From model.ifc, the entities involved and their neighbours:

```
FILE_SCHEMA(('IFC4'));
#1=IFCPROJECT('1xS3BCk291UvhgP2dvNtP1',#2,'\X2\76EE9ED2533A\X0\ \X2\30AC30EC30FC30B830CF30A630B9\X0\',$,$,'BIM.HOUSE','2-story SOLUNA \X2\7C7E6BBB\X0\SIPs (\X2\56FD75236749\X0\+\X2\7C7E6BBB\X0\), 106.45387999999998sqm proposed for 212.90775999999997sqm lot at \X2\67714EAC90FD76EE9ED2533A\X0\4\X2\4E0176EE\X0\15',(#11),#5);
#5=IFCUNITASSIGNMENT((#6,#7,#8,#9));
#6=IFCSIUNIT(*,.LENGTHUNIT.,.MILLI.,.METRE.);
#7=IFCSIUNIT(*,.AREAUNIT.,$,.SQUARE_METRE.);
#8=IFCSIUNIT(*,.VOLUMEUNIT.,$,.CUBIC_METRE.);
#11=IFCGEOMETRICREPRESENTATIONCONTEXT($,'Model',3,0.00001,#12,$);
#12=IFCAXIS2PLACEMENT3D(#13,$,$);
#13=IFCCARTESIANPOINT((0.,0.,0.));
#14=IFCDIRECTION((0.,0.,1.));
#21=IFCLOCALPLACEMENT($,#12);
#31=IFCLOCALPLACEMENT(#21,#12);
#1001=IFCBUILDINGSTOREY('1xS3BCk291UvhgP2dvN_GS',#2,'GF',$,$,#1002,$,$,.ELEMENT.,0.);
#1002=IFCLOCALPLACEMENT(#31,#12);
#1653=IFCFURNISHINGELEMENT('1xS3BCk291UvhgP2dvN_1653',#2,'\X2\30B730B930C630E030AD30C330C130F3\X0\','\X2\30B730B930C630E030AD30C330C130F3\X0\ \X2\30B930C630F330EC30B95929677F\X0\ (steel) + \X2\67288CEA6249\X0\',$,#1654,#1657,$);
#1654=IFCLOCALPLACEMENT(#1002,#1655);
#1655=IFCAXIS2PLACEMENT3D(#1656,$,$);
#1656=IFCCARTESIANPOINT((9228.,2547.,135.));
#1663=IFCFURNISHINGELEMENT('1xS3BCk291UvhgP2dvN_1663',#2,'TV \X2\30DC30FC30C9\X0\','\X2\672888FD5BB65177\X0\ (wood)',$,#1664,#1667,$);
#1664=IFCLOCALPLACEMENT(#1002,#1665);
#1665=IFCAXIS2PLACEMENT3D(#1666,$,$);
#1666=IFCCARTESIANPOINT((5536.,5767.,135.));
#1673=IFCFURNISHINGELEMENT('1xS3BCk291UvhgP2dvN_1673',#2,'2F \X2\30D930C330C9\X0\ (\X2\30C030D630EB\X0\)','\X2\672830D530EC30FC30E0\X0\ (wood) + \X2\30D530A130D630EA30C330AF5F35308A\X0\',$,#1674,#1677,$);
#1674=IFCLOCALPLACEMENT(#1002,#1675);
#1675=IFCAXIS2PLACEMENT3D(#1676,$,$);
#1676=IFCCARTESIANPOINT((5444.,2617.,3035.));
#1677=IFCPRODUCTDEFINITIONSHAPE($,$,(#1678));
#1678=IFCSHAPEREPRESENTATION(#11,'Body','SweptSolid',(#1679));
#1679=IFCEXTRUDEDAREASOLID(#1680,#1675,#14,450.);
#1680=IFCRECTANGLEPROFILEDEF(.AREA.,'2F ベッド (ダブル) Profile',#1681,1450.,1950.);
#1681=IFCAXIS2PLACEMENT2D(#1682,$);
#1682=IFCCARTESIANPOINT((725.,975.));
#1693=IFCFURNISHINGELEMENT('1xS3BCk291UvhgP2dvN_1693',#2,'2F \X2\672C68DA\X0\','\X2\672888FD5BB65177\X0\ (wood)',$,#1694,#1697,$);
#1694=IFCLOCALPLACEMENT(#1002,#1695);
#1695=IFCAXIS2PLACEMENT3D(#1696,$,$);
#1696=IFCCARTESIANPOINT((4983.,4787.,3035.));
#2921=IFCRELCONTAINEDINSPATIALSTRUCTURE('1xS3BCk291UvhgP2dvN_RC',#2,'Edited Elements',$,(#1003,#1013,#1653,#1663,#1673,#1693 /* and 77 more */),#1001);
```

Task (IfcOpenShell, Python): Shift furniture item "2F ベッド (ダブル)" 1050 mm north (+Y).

```python
import ifcopenshell
import ifcopenshell.api.geometry
import ifcopenshell.util.placement
import ifcopenshell.util.unit

model = ifcopenshell.open("model.ifc")
unit_scale = ifcopenshell.util.unit.calculate_unit_scale(model)

item = model.by_guid("1xS3BCk291UvhgP2dvN_1673")
matrix = ifcopenshell.util.placement.get_local_placement(item.ObjectPlacement)
matrix[1, 3] += 1.05 / unit_scale
ifcopenshell.api.geometry.edit_object_placement(model, product=item, matrix=matrix, is_si=False)

print(ifcopenshell.util.placement.get_local_placement(item.ObjectPlacement).round(3) + 0.0)

model.write("model-out.ifc")
```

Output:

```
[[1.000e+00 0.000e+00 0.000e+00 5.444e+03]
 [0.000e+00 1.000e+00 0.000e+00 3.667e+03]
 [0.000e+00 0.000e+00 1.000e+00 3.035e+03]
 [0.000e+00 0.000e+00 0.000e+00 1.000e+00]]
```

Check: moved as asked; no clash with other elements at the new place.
